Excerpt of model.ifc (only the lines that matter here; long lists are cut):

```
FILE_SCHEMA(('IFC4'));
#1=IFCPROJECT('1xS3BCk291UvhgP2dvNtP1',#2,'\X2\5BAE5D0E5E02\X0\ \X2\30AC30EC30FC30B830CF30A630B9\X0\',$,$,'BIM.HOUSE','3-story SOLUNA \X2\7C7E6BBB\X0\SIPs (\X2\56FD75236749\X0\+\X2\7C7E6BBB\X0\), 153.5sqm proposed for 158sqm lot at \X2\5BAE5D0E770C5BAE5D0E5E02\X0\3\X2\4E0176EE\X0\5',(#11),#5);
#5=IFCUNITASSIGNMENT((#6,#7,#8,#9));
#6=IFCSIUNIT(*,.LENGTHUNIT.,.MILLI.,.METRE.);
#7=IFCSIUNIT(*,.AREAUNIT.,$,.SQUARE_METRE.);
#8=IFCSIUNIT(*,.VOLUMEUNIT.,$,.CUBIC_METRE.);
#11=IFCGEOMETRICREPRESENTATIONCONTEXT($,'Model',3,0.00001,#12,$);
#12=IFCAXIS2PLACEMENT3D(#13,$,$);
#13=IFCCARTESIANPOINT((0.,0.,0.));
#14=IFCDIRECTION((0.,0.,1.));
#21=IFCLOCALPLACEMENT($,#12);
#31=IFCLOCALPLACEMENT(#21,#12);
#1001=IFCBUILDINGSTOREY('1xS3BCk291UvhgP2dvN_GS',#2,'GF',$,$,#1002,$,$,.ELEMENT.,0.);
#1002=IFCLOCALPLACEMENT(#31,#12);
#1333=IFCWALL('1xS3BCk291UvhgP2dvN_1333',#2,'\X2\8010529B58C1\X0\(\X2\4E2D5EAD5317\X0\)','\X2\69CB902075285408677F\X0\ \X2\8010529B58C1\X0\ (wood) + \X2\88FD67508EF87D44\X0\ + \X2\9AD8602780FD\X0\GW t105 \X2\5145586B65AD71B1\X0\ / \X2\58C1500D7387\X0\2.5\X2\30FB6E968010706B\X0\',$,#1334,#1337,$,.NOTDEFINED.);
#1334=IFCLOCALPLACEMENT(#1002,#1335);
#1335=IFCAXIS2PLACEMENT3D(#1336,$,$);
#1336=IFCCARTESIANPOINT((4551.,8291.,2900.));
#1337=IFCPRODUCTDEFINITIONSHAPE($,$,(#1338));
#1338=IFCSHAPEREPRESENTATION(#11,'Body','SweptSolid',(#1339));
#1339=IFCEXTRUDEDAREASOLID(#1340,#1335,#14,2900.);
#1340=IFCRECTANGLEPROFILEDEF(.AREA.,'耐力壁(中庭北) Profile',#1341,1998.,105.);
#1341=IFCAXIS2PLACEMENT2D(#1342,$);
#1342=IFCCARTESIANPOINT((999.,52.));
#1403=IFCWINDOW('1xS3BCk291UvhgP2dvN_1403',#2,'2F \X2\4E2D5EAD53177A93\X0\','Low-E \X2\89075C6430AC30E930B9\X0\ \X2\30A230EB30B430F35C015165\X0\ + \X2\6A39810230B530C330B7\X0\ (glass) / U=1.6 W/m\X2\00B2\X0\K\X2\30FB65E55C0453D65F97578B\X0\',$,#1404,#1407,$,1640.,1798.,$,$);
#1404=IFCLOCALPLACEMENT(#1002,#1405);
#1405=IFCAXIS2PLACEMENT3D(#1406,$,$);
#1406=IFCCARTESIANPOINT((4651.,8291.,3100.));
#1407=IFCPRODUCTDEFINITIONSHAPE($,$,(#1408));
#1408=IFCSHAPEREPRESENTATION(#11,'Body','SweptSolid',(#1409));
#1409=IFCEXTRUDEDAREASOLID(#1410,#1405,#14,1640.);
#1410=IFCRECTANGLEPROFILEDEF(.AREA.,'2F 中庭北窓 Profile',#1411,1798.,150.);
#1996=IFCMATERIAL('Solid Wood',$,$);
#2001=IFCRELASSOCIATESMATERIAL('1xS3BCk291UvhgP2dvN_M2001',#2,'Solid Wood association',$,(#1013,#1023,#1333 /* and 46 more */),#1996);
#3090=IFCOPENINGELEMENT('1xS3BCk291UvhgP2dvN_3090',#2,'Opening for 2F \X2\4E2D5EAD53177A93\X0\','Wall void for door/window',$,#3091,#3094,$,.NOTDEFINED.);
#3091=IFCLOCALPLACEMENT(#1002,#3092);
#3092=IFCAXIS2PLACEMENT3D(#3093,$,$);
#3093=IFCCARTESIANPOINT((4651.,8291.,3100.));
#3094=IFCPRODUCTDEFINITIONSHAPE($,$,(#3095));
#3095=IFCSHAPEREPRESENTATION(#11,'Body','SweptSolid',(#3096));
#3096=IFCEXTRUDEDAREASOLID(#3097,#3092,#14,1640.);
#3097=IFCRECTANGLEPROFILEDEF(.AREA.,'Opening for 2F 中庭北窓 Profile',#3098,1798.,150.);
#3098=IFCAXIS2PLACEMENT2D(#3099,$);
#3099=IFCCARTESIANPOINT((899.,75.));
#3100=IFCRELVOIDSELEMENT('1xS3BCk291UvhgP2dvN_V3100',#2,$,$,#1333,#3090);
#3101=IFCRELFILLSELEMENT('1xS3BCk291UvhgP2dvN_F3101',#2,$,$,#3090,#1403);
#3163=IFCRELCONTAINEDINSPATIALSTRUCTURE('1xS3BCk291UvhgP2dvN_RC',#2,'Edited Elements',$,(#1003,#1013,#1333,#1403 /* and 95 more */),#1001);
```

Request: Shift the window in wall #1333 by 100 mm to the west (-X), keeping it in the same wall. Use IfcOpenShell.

```python
import ifcopenshell
import ifcopenshell.api.geometry
import ifcopenshell.util.placement
import ifcopenshell.util.unit

model = ifcopenshell.open("model.ifc")
unit_scale = ifcopenshell.util.unit.calculate_unit_scale(model)

window = model.by_guid("1xS3BCk291UvhgP2dvN_1403")
opening = window.FillsVoids[0].RelatingOpeningElement
wall = opening.VoidsElements[0].RelatingBuildingElement

wall_matrix = ifcopenshell.util.placement.get_local_placement(wall.ObjectPlacement)
shift = wall_matrix[:3, 0] * -0.1 / unit_scale
before = ifcopenshell.util.placement.get_local_placement(window.ObjectPlacement)[:3, 3].copy()

# The window is not placed relative to its opening, so move both.
for product in (opening, window):
    matrix = ifcopenshell.util.placement.get_local_placement(product.ObjectPlacement)
    matrix[:3, 3] += shift
    ifcopenshell.api.geometry.edit_object_placement(model, product=product, matrix=matrix, is_si=False)

after = ifcopenshell.util.placement.get_local_placement(window.ObjectPlacement)[:3, 3]
print("window moved by", (after - before).round(3) + 0.0)

model.write("model_rev.ifc")
```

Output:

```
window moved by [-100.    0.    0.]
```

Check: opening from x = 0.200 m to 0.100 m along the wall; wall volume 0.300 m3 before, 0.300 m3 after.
